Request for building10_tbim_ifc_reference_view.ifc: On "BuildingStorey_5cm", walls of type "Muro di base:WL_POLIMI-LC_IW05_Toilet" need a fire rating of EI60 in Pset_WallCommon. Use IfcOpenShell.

First a look at what the model holds.

```python
import ifcopenshell
import ifcopenshell.util.element

model = ifcopenshell.open("building10_tbim_ifc_reference_view.ifc")
print(model.schema)
storey = next(s for s in model.by_type("IfcBuildingStorey") if s.Name == "BuildingStorey_5cm")
walls = [e for e in ifcopenshell.util.element.get_decomposition(storey) if e.is_a("IfcWall")]
seen = {}
for e in walls:
    element_type = ifcopenshell.util.element.get_type(e)
    key = (element_type.Name if element_type != e and element_type else None, ifcopenshell.util.element.get_pset(e, "Pset_WallCommon", "FireRating"))
    seen[key] = seen.get(key, 0) + 1
for (name, value), count in sorted(seen.items(), key=str):
    print(count, "x", name, "|", value)
```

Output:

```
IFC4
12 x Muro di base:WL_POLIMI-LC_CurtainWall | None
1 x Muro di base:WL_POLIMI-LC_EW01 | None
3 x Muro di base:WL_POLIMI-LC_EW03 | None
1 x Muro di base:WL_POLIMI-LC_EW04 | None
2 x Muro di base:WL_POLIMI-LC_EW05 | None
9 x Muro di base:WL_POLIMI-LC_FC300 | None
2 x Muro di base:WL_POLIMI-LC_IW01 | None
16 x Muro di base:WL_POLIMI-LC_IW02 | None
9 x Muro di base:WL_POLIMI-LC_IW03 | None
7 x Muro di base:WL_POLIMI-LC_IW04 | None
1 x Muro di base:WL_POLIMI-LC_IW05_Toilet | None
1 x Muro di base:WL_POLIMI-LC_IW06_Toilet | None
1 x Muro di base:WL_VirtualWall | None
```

```python
import ifcopenshell
import ifcopenshell.api.pset
import ifcopenshell.util.element

model = ifcopenshell.open("building10_tbim_ifc_reference_view.ifc")

storey = next(s for s in model.by_type("IfcBuildingStorey") if s.Name == "BuildingStorey_5cm")
walls = [e for e in ifcopenshell.util.element.get_decomposition(storey) if e.is_a("IfcWall")]

count = 0
for e in walls:
    element_type = ifcopenshell.util.element.get_type(e)
    if element_type in (None, e) or element_type.Name != "Muro di base:WL_POLIMI-LC_IW05_Toilet":
        continue
    # add_pset returns the element's existing set when there is one.
    pset = ifcopenshell.api.pset.add_pset(model, product=e, name="Pset_WallCommon")
    ifcopenshell.api.pset.edit_pset(model, pset=pset, properties={"FireRating": "EI60"})
    count += 1

print(count, "walls updated")

model.write("building10_tbim_ifc_reference_view_v2.ifc")
```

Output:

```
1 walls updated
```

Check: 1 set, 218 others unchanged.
